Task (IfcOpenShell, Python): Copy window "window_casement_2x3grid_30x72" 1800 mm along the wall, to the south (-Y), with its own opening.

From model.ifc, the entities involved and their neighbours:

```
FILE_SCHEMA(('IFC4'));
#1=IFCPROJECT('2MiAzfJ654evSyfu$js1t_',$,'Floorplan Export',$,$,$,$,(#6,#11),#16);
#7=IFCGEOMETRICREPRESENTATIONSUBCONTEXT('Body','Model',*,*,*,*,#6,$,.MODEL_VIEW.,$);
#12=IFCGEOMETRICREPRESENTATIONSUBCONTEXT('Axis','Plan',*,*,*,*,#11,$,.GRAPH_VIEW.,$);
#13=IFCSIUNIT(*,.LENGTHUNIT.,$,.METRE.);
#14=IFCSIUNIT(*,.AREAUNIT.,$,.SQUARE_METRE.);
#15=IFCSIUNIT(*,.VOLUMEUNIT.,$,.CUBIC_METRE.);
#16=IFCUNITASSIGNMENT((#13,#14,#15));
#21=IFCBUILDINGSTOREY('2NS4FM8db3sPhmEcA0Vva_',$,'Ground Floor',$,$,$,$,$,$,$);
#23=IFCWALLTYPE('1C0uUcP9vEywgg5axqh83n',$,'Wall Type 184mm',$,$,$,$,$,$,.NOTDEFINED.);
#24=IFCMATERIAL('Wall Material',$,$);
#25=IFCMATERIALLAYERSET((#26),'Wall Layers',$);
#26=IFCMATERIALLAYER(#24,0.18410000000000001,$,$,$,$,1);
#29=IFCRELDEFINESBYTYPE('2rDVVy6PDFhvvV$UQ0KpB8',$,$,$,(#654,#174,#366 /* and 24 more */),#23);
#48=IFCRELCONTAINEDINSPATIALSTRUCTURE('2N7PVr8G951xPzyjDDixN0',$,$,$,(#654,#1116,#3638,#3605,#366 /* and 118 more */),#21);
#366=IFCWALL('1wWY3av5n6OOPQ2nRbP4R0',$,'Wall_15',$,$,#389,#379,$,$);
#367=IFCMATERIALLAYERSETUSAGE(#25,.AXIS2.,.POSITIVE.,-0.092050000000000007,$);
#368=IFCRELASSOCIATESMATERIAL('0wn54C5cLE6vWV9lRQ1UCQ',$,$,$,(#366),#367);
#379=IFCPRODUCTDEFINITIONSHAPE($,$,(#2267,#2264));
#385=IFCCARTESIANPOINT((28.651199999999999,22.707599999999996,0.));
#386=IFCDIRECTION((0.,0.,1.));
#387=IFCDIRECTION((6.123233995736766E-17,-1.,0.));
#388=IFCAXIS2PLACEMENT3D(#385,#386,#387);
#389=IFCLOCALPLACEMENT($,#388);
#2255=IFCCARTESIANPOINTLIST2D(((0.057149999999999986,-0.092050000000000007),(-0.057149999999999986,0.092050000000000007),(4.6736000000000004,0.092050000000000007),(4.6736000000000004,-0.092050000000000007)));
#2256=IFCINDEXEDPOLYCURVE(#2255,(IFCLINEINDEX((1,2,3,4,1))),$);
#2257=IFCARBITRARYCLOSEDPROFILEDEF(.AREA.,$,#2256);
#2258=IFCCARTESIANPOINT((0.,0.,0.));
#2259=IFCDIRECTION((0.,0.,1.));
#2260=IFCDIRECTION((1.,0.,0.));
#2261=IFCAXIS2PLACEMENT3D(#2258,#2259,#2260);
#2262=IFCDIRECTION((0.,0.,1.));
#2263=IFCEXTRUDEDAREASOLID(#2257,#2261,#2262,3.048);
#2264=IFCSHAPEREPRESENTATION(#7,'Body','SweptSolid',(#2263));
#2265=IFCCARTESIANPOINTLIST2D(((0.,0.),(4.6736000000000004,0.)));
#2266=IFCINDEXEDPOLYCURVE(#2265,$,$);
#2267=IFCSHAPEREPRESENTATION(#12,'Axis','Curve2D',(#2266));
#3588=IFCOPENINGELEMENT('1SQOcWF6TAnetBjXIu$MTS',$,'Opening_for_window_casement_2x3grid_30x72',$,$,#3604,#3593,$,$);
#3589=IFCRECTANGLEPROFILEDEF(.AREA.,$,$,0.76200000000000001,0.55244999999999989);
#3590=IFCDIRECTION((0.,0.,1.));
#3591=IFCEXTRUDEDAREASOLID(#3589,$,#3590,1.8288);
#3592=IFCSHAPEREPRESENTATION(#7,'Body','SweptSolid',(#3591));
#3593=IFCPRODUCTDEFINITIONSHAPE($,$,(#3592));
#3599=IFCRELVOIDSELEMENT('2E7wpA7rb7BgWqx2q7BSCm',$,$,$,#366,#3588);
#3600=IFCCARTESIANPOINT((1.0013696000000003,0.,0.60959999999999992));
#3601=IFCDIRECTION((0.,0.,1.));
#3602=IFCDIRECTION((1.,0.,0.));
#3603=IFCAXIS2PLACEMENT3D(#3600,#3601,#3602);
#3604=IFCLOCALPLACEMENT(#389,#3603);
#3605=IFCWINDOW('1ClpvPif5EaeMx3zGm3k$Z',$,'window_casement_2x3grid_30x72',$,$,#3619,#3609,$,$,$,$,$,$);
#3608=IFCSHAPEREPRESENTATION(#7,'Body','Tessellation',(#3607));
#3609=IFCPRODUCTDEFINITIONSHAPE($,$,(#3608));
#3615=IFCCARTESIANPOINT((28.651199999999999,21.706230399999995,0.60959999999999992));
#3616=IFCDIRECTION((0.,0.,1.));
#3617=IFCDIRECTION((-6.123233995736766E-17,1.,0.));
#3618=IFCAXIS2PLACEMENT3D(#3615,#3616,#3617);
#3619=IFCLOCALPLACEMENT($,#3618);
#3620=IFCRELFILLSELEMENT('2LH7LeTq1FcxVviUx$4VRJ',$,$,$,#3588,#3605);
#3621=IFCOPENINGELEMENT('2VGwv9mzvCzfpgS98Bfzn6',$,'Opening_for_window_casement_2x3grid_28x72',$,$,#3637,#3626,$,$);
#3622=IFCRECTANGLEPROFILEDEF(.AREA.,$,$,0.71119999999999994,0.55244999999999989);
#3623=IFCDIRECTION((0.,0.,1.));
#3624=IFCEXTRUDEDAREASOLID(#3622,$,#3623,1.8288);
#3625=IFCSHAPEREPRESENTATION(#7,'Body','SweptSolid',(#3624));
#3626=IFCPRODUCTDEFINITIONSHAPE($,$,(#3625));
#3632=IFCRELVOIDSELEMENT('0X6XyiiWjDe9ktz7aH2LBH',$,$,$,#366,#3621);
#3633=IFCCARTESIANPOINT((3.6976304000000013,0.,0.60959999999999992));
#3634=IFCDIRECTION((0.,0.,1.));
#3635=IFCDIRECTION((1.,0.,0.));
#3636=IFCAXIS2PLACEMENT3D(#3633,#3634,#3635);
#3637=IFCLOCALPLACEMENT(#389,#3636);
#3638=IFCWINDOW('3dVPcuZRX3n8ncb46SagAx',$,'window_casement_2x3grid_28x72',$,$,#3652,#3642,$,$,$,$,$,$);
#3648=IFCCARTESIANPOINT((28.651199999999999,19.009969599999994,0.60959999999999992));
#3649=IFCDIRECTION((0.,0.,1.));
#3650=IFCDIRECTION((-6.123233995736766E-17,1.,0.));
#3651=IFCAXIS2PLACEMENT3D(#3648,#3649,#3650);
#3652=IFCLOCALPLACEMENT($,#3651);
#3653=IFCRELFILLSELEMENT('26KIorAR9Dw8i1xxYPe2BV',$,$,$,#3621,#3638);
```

```python
import ifcopenshell
import ifcopenshell.api.feature
import ifcopenshell.api.geometry
import ifcopenshell.api.root
import ifcopenshell.geom
import ifcopenshell.util.element
import ifcopenshell.util.placement
import ifcopenshell.util.shape
import ifcopenshell.util.unit

model = ifcopenshell.open("model.ifc")
unit_scale = ifcopenshell.util.unit.calculate_unit_scale(model)
settings = ifcopenshell.geom.settings()


def volume(element):
    """Net volume in cubic metres, openings subtracted."""
    shape = ifcopenshell.geom.create_shape(settings, element)
    return ifcopenshell.util.shape.get_volume(shape.geometry)


window = model.by_guid("1ClpvPif5EaeMx3zGm3k$Z")
opening = window.FillsVoids[0].RelatingOpeningElement
wall = opening.VoidsElements[0].RelatingBuildingElement
before = volume(wall)
shift = ifcopenshell.util.placement.get_local_placement(wall.ObjectPlacement)[:3, 0] * 1.8 / unit_scale

# copy_class copies the void relationship, type, container and properties, but no geometry.
new_opening = ifcopenshell.api.root.copy_class(model, product=opening)
new_opening.Representation = ifcopenshell.util.element.copy_deep(
    model, opening.Representation, exclude=["IfcGeometricRepresentationContext", "IfcRepresentationMap"]
)
new_window = ifcopenshell.api.root.copy_class(model, product=window)
new_window.Representation = ifcopenshell.util.element.copy_deep(
    model, window.Representation, exclude=["IfcGeometricRepresentationContext", "IfcRepresentationMap"]
)
ifcopenshell.api.feature.add_filling(model, opening=new_opening, element=new_window)

for old, new in ((opening, new_opening), (window, new_window)):
    matrix = ifcopenshell.util.placement.get_local_placement(old.ObjectPlacement)
    matrix[:3, 3] += shift
    ifcopenshell.api.geometry.edit_object_placement(model, product=new, matrix=matrix, is_si=False)

after = volume(wall)

print(f"wall volume {before:.3f} -> {after:.3f} m3")

model.write("model_v2.ifc")
```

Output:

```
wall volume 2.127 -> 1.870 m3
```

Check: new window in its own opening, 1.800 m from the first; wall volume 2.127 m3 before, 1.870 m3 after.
